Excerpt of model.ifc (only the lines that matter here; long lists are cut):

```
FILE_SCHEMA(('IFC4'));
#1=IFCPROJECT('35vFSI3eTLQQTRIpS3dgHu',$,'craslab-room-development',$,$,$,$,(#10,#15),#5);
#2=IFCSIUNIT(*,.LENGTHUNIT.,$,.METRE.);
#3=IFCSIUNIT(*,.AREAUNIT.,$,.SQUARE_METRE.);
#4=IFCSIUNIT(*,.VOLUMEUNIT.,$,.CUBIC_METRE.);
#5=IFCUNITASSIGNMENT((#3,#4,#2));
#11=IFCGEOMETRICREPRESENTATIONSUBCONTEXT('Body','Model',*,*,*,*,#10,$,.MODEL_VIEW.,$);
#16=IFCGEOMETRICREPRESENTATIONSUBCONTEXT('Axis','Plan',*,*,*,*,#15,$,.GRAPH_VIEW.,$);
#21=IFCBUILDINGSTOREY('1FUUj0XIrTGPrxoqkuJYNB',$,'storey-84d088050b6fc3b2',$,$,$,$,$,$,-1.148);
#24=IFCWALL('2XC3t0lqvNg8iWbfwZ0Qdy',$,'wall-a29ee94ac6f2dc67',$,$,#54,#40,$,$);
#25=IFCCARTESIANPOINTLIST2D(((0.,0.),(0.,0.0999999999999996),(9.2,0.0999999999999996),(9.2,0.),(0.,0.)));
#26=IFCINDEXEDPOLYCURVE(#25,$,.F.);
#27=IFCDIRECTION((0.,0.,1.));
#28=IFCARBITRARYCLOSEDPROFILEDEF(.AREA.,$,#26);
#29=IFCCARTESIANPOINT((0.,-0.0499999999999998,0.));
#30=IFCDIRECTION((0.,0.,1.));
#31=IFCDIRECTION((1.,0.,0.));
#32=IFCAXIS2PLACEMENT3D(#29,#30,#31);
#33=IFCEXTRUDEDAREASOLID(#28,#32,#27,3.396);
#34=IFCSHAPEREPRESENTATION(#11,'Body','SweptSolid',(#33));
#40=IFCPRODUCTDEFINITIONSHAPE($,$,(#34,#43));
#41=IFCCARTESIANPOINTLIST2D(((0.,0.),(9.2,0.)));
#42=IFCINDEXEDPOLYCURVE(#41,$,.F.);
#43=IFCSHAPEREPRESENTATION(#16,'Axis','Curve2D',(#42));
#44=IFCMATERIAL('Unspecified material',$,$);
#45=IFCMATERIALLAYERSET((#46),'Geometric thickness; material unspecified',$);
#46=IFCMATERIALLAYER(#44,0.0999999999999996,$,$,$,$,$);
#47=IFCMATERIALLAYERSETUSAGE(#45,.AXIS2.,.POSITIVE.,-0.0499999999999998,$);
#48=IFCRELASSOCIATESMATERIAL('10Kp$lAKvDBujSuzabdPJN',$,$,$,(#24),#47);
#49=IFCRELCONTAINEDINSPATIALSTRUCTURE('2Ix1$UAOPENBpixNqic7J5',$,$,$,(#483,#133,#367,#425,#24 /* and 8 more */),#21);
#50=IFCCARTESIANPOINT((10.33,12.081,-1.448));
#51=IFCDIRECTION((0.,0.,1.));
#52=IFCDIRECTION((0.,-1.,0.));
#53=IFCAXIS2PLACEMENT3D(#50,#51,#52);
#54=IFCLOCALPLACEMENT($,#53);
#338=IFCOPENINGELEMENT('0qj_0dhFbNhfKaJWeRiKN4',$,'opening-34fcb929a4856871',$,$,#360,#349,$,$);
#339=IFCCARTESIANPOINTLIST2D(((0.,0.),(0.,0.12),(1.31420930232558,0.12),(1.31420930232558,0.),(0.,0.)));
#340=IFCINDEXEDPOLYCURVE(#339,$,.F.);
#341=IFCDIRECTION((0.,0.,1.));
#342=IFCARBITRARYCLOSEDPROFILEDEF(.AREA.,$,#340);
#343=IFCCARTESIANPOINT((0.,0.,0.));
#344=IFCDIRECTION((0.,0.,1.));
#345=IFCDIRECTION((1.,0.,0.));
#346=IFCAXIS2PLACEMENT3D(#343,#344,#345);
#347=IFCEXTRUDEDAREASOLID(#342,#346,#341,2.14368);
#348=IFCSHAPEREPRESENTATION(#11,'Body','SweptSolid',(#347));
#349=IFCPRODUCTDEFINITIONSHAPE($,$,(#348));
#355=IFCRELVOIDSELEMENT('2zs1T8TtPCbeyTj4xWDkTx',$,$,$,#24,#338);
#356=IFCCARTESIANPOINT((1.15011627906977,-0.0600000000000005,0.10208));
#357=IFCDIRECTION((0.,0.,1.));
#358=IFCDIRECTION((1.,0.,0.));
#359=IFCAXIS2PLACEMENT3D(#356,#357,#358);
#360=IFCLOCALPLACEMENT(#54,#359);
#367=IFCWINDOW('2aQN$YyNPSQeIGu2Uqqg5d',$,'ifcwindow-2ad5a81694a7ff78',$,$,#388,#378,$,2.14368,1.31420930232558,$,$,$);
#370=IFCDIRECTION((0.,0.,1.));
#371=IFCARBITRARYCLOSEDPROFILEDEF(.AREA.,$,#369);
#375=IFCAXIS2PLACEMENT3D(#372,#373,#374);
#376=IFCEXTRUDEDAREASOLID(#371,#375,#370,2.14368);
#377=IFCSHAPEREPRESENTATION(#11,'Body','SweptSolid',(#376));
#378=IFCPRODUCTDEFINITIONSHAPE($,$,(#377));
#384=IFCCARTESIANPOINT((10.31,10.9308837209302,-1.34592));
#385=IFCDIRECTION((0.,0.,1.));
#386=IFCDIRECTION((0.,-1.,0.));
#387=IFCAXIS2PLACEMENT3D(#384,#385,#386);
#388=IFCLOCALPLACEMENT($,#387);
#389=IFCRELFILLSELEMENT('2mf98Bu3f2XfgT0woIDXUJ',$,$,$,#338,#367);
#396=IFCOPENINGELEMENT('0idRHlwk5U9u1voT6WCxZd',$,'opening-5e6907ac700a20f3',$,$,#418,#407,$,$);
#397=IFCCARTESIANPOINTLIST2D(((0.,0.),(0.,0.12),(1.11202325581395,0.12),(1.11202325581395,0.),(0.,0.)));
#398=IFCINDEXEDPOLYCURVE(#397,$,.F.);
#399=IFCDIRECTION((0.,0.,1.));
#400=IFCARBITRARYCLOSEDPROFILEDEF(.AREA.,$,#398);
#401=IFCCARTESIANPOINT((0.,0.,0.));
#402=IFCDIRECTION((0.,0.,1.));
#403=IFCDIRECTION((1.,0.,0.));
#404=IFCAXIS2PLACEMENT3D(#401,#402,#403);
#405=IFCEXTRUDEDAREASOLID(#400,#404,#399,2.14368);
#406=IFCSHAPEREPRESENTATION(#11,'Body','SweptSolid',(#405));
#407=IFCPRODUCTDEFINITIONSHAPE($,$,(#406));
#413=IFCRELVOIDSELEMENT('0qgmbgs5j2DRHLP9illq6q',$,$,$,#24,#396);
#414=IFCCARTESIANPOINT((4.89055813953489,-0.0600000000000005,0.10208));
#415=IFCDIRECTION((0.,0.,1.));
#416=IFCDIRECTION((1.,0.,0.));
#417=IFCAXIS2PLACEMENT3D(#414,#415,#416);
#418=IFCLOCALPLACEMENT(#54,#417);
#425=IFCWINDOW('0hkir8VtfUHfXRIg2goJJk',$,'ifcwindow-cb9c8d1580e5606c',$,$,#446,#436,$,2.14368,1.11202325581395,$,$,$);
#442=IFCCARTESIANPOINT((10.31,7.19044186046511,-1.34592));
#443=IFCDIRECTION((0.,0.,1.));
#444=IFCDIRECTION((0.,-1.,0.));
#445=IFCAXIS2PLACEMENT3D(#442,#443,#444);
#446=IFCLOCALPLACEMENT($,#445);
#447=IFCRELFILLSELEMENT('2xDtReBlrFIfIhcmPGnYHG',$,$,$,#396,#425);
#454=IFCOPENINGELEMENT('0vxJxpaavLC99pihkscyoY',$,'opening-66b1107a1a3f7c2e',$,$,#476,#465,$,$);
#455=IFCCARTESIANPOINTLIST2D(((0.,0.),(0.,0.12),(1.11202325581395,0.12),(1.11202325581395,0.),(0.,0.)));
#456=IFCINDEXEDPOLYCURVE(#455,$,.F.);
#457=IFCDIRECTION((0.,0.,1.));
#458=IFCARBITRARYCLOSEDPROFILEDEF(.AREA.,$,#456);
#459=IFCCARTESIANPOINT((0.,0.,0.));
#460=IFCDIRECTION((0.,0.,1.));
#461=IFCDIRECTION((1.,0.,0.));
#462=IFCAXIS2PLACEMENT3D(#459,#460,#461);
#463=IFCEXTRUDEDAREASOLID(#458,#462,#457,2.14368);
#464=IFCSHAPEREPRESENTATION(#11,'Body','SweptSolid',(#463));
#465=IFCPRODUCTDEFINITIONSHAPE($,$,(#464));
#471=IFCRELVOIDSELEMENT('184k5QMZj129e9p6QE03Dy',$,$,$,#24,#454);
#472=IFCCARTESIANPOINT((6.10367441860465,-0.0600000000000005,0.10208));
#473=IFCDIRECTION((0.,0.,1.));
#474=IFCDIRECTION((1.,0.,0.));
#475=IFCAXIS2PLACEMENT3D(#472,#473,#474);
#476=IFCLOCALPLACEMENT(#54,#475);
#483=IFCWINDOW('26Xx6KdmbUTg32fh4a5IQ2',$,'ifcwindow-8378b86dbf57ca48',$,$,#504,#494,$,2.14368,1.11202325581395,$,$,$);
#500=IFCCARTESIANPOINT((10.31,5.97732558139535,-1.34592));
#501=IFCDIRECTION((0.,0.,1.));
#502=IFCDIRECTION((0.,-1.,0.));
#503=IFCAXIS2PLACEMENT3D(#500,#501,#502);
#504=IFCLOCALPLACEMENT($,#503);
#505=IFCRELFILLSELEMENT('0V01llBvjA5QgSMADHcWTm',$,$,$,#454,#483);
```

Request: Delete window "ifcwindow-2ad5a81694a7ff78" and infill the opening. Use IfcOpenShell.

```python
import ifcopenshell
import ifcopenshell.api.feature
import ifcopenshell.api.root
import ifcopenshell.geom
import ifcopenshell.util.shape

model = ifcopenshell.open("model.ifc")
settings = ifcopenshell.geom.settings()


def volume(element):
    """Net volume in cubic metres, openings subtracted."""
    shape = ifcopenshell.geom.create_shape(settings, element)
    return ifcopenshell.util.shape.get_volume(shape.geometry)


window = model.by_id(367)
opening = window.FillsVoids[0].RelatingOpeningElement
wall = opening.VoidsElements[0].RelatingBuildingElement
before = volume(wall)

ifcopenshell.api.root.remove_product(model, product=window)
ifcopenshell.api.feature.remove_feature(model, feature=opening)

after = volume(wall)

print(f"wall volume {before:.3f} -> {after:.3f} m3")

model.write("model_v2.ifc")
```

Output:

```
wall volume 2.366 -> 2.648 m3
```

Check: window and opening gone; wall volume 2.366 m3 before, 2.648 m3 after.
